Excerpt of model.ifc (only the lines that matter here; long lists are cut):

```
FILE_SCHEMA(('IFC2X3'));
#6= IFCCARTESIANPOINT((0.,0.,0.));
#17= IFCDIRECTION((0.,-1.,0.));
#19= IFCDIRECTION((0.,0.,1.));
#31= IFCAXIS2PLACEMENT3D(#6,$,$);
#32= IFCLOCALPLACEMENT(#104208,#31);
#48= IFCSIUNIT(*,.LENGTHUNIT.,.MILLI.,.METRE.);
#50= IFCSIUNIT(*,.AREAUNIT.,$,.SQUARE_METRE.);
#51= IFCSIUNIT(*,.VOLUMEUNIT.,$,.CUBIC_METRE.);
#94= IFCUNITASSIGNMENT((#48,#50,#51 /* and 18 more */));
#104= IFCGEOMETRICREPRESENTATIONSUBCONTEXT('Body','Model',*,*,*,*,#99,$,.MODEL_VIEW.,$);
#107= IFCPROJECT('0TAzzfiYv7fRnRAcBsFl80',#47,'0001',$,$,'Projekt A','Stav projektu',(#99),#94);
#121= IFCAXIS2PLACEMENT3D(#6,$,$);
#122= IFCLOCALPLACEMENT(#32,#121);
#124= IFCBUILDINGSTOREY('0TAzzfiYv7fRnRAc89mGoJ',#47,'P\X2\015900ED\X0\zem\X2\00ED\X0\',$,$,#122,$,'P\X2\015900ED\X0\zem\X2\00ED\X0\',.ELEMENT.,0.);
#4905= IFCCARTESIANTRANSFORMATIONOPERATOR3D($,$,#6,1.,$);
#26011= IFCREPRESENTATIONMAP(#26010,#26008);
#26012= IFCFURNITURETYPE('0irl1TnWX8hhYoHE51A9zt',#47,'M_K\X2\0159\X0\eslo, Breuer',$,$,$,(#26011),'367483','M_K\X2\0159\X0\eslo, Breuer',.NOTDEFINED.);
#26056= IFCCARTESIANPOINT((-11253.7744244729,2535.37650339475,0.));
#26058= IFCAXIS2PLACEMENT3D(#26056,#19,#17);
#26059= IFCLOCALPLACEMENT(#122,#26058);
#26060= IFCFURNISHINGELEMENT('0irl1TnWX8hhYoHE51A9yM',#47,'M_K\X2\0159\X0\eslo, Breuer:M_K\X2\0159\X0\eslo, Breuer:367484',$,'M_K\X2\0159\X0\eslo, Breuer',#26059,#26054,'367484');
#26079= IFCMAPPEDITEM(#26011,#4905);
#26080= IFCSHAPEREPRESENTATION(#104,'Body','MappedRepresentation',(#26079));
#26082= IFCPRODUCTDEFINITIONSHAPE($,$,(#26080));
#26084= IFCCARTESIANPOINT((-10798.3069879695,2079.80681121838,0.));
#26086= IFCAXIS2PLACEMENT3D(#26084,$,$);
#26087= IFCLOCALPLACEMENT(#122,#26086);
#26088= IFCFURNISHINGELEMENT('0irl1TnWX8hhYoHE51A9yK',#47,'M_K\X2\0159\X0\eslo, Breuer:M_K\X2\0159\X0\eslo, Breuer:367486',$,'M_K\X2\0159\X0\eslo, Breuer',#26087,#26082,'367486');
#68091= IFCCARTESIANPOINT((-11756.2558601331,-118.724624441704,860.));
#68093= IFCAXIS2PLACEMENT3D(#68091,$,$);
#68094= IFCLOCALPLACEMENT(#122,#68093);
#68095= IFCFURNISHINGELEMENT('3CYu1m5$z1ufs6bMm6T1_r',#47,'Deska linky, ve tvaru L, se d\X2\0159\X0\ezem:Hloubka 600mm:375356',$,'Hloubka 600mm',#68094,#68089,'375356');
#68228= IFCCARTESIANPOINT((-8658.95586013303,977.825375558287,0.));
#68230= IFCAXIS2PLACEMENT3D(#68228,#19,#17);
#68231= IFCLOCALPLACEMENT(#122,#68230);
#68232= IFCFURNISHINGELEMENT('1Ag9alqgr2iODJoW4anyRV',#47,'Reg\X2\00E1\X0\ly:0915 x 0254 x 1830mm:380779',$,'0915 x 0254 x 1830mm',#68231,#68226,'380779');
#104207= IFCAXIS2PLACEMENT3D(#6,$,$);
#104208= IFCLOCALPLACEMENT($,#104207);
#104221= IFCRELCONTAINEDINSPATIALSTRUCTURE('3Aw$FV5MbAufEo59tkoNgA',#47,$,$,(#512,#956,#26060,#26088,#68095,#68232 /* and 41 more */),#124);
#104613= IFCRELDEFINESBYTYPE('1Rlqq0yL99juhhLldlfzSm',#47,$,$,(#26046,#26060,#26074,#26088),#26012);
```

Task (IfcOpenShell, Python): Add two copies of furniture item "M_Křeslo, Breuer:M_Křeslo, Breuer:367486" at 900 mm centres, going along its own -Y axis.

```python
import ifcopenshell
import ifcopenshell.api.geometry
import ifcopenshell.api.root
import ifcopenshell.util.element
import ifcopenshell.util.placement

model = ifcopenshell.open("model.ifc")

source = model.by_guid("0irl1TnWX8hhYoHE51A9yK")
base = ifcopenshell.util.placement.get_local_placement(source.ObjectPlacement)
step = -base[:3, 1] * 900.0

for i in range(1, 3):
    copy = ifcopenshell.api.root.copy_class(model, product=source)
    copy.Representation = ifcopenshell.util.element.copy_deep(
        model, source.Representation, exclude=["IfcGeometricRepresentationContext", "IfcRepresentationMap"]
    )
    copy.Name = "M_Křeslo, Breuer:M_Křeslo, Breuer"
    copy.Tag = None
    matrix = base.copy()
    matrix[:3, 3] += i * step
    print("added at", matrix[:3, 3].round(3) + 0.0)
    ifcopenshell.api.geometry.edit_object_placement(model, product=copy, matrix=matrix, is_si=False)

model.write("model_edited.ifc")
```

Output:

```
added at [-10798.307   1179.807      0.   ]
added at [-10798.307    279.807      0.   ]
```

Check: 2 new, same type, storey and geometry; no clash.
